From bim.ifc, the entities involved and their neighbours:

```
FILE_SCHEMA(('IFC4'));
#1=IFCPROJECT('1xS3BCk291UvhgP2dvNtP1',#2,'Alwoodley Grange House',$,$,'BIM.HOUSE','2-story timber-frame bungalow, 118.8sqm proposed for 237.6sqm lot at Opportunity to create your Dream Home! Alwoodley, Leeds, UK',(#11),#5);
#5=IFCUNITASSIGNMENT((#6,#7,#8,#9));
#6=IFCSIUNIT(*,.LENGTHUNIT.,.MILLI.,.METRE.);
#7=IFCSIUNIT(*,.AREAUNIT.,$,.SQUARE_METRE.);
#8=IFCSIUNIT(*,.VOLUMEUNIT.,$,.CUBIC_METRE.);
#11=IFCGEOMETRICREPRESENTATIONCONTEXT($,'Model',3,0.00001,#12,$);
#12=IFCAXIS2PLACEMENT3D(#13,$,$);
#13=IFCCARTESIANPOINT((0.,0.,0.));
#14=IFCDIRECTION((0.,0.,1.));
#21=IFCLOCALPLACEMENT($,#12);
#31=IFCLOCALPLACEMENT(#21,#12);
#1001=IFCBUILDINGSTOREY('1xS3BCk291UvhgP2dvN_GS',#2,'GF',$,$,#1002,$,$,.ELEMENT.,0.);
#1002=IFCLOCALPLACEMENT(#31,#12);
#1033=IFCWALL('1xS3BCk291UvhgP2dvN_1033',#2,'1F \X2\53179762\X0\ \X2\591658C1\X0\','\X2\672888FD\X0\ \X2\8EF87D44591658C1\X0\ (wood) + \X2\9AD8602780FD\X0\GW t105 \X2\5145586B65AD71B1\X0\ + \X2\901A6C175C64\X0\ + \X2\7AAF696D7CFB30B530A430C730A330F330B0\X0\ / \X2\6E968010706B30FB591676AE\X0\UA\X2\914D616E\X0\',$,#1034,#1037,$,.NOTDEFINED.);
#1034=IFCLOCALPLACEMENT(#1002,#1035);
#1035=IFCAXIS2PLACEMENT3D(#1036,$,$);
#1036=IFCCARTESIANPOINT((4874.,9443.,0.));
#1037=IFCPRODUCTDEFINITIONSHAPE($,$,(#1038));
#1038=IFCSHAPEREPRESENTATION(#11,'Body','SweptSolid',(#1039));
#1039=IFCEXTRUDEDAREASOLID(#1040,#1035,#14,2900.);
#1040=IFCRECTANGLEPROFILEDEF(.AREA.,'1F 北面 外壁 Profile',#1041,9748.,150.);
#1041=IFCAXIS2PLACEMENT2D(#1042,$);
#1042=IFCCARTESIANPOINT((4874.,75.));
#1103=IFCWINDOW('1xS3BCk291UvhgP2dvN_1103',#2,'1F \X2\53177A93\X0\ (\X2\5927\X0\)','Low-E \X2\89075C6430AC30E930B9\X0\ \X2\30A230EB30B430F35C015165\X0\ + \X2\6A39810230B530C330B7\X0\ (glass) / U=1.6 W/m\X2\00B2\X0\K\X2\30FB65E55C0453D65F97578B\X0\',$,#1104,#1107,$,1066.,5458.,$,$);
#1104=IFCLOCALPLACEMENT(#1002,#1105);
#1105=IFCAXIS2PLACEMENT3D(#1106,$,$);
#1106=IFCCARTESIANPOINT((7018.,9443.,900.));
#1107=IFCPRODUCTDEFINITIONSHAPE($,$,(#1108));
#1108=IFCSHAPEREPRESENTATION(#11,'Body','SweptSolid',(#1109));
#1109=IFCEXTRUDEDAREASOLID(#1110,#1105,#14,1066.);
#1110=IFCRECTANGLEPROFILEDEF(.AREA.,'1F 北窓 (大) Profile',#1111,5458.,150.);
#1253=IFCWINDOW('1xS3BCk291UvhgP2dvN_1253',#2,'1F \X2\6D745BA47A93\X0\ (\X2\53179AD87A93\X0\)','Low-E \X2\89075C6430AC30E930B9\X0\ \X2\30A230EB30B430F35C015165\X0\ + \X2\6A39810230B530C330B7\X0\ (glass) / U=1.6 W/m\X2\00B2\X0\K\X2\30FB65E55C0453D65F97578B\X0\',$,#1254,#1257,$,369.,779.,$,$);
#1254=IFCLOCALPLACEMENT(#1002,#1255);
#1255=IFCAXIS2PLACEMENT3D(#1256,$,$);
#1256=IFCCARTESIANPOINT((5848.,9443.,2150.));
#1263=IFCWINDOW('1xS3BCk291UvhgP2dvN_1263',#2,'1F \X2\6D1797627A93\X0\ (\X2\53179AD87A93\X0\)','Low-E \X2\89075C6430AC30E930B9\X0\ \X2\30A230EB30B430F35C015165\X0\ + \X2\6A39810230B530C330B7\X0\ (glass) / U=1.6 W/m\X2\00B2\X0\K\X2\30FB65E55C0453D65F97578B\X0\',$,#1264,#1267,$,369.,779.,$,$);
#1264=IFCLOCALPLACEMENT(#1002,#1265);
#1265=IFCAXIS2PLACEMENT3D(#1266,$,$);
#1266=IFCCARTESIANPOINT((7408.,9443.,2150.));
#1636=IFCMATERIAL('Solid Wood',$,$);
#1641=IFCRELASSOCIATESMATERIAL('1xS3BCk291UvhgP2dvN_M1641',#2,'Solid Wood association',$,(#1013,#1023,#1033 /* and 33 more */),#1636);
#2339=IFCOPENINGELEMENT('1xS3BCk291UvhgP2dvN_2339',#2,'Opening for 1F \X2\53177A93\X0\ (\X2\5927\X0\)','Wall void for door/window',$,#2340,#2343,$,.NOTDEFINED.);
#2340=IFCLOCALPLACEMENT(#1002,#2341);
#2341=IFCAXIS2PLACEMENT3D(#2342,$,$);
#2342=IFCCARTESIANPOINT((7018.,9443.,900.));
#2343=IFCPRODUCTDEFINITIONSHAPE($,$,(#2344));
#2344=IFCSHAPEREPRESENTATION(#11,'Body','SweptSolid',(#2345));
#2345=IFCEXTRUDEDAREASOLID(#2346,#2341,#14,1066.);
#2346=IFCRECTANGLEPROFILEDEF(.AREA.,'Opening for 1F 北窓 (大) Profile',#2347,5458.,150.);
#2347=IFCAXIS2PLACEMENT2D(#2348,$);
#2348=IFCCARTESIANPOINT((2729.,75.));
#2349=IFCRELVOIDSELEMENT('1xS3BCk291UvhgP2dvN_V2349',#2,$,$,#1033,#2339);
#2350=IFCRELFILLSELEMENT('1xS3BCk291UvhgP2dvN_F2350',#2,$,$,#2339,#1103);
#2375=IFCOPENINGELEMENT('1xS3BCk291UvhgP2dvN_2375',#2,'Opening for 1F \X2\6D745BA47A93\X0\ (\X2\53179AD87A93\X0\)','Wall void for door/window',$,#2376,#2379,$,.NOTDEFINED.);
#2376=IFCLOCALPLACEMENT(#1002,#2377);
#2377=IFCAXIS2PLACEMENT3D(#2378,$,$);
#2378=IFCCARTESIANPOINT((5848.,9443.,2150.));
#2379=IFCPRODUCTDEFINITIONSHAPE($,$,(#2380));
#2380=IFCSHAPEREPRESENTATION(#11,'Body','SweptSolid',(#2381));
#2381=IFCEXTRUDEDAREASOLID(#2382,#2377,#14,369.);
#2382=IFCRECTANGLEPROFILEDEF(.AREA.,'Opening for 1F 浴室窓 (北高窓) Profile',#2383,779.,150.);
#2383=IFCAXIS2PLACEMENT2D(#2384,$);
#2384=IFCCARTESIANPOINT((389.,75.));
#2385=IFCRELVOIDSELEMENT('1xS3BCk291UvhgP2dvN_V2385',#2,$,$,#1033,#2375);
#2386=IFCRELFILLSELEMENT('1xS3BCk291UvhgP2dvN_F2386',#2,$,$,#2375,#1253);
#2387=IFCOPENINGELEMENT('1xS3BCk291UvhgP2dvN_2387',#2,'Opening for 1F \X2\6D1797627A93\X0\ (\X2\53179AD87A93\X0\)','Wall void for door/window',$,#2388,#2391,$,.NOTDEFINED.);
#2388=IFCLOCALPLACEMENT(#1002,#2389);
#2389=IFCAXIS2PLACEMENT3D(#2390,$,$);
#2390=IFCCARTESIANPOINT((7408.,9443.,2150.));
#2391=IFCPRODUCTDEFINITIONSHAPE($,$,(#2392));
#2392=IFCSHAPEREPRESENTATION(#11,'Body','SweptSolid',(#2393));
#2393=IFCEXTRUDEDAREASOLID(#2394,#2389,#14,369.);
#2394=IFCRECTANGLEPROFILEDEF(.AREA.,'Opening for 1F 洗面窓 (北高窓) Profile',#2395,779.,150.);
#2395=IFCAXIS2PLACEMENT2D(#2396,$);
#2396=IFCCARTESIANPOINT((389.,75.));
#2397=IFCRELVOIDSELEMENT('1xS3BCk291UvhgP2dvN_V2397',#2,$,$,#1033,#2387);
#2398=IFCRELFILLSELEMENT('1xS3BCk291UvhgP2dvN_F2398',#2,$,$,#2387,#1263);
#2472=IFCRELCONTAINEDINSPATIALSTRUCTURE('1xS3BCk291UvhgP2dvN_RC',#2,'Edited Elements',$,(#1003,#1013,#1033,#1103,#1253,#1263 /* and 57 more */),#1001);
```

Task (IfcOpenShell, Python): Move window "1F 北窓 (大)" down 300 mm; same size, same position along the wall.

```python
import numpy as np
import ifcopenshell
import ifcopenshell.api.geometry
import ifcopenshell.util.placement
import ifcopenshell.util.unit

model = ifcopenshell.open("bim.ifc")
unit_scale = ifcopenshell.util.unit.calculate_unit_scale(model)

window = model.by_guid("1xS3BCk291UvhgP2dvN_1103")
opening = window.FillsVoids[0].RelatingOpeningElement
dz = -300.0

shift = np.array([0.0, 0.0, dz])
# The window is not placed relative to its opening, so move both.
for product in (opening, window):
    matrix = ifcopenshell.util.placement.get_local_placement(product.ObjectPlacement)
    matrix[:3, 3] += shift
    ifcopenshell.api.geometry.edit_object_placement(model, product=product, matrix=matrix, is_si=False)

print(f"moved by {dz * unit_scale:+.3f} m")

model.write("bim_updated.ifc")
```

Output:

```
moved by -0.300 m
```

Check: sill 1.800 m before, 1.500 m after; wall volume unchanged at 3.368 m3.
